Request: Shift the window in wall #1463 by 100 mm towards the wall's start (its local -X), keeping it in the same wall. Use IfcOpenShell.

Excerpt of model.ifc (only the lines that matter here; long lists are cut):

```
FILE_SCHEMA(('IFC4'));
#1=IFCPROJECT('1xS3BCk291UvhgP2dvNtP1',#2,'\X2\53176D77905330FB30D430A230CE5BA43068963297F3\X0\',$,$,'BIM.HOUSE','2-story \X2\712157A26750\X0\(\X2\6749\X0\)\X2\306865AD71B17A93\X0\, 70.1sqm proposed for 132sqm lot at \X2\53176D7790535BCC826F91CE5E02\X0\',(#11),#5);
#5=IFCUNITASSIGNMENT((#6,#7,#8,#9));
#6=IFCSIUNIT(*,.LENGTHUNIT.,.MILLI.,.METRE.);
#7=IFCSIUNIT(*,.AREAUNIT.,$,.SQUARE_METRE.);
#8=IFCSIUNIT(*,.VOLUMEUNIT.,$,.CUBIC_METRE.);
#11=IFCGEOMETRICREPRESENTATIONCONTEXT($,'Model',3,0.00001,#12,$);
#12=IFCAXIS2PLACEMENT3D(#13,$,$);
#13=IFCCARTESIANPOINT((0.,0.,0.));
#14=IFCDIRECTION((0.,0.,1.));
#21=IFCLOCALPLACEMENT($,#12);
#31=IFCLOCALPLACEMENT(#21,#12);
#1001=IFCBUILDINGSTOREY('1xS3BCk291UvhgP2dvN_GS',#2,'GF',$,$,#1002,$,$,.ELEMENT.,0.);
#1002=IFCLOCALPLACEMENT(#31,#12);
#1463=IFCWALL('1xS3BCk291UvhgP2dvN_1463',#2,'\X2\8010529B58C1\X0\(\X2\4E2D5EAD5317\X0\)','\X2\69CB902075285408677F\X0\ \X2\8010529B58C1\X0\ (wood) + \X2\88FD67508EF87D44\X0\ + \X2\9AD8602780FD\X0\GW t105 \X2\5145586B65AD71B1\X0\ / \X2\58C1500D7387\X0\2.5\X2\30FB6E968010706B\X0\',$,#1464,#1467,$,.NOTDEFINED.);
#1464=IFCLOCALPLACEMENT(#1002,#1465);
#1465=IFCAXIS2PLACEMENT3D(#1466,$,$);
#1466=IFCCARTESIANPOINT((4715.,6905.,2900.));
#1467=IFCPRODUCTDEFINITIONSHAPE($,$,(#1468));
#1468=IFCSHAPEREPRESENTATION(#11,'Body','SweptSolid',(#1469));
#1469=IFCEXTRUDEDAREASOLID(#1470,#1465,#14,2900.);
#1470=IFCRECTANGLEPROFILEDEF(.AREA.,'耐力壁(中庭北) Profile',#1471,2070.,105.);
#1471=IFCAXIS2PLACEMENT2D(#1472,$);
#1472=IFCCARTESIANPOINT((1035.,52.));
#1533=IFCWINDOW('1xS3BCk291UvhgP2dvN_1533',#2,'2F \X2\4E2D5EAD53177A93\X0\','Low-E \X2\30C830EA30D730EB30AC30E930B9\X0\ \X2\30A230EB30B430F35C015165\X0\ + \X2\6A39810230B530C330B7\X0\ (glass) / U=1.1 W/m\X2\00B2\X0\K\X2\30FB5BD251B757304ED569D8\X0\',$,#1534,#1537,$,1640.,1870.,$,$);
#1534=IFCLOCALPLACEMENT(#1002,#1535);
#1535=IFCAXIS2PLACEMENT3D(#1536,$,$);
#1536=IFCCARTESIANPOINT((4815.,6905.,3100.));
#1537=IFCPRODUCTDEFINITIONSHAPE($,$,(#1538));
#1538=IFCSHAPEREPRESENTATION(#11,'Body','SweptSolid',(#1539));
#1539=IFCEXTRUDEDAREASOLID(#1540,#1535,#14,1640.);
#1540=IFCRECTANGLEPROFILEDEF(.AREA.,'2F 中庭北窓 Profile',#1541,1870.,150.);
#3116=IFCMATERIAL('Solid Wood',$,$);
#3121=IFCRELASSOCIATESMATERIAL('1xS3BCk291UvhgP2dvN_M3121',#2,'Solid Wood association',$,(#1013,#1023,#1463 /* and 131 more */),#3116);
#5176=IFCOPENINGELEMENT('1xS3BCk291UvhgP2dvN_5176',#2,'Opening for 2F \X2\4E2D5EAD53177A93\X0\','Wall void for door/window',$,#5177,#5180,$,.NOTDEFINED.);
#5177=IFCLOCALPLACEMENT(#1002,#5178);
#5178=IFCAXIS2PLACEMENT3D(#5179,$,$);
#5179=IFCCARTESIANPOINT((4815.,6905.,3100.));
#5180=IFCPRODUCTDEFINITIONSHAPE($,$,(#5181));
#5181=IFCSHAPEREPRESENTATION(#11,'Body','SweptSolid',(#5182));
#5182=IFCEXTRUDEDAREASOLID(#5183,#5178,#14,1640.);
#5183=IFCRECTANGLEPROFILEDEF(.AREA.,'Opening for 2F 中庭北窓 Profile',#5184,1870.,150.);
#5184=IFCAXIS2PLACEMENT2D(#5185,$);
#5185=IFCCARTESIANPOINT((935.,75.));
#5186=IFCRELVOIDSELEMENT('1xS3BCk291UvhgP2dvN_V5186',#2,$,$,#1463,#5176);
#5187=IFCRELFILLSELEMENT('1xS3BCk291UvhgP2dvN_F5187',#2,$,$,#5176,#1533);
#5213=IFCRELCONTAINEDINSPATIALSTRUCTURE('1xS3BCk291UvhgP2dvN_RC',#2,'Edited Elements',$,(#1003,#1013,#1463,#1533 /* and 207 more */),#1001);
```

```python
import ifcopenshell
import ifcopenshell.api.geometry
import ifcopenshell.util.placement
import ifcopenshell.util.unit

model = ifcopenshell.open("model.ifc")
unit_scale = ifcopenshell.util.unit.calculate_unit_scale(model)

window = model.by_guid("1xS3BCk291UvhgP2dvN_1533")
opening = window.FillsVoids[0].RelatingOpeningElement
wall = opening.VoidsElements[0].RelatingBuildingElement

wall_matrix = ifcopenshell.util.placement.get_local_placement(wall.ObjectPlacement)
shift = wall_matrix[:3, 0] * -0.1 / unit_scale
before = ifcopenshell.util.placement.get_local_placement(window.ObjectPlacement)[:3, 3].copy()

# The window is not placed relative to its opening, so move both.
for product in (opening, window):
    matrix = ifcopenshell.util.placement.get_local_placement(product.ObjectPlacement)
    matrix[:3, 3] += shift
    ifcopenshell.api.geometry.edit_object_placement(model, product=product, matrix=matrix, is_si=False)

after = ifcopenshell.util.placement.get_local_placement(window.ObjectPlacement)[:3, 3]
print("window moved by", (after - before).round(3) + 0.0)

model.write("model_updated.ifc")
```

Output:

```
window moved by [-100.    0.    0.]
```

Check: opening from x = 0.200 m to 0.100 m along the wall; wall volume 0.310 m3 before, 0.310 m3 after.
